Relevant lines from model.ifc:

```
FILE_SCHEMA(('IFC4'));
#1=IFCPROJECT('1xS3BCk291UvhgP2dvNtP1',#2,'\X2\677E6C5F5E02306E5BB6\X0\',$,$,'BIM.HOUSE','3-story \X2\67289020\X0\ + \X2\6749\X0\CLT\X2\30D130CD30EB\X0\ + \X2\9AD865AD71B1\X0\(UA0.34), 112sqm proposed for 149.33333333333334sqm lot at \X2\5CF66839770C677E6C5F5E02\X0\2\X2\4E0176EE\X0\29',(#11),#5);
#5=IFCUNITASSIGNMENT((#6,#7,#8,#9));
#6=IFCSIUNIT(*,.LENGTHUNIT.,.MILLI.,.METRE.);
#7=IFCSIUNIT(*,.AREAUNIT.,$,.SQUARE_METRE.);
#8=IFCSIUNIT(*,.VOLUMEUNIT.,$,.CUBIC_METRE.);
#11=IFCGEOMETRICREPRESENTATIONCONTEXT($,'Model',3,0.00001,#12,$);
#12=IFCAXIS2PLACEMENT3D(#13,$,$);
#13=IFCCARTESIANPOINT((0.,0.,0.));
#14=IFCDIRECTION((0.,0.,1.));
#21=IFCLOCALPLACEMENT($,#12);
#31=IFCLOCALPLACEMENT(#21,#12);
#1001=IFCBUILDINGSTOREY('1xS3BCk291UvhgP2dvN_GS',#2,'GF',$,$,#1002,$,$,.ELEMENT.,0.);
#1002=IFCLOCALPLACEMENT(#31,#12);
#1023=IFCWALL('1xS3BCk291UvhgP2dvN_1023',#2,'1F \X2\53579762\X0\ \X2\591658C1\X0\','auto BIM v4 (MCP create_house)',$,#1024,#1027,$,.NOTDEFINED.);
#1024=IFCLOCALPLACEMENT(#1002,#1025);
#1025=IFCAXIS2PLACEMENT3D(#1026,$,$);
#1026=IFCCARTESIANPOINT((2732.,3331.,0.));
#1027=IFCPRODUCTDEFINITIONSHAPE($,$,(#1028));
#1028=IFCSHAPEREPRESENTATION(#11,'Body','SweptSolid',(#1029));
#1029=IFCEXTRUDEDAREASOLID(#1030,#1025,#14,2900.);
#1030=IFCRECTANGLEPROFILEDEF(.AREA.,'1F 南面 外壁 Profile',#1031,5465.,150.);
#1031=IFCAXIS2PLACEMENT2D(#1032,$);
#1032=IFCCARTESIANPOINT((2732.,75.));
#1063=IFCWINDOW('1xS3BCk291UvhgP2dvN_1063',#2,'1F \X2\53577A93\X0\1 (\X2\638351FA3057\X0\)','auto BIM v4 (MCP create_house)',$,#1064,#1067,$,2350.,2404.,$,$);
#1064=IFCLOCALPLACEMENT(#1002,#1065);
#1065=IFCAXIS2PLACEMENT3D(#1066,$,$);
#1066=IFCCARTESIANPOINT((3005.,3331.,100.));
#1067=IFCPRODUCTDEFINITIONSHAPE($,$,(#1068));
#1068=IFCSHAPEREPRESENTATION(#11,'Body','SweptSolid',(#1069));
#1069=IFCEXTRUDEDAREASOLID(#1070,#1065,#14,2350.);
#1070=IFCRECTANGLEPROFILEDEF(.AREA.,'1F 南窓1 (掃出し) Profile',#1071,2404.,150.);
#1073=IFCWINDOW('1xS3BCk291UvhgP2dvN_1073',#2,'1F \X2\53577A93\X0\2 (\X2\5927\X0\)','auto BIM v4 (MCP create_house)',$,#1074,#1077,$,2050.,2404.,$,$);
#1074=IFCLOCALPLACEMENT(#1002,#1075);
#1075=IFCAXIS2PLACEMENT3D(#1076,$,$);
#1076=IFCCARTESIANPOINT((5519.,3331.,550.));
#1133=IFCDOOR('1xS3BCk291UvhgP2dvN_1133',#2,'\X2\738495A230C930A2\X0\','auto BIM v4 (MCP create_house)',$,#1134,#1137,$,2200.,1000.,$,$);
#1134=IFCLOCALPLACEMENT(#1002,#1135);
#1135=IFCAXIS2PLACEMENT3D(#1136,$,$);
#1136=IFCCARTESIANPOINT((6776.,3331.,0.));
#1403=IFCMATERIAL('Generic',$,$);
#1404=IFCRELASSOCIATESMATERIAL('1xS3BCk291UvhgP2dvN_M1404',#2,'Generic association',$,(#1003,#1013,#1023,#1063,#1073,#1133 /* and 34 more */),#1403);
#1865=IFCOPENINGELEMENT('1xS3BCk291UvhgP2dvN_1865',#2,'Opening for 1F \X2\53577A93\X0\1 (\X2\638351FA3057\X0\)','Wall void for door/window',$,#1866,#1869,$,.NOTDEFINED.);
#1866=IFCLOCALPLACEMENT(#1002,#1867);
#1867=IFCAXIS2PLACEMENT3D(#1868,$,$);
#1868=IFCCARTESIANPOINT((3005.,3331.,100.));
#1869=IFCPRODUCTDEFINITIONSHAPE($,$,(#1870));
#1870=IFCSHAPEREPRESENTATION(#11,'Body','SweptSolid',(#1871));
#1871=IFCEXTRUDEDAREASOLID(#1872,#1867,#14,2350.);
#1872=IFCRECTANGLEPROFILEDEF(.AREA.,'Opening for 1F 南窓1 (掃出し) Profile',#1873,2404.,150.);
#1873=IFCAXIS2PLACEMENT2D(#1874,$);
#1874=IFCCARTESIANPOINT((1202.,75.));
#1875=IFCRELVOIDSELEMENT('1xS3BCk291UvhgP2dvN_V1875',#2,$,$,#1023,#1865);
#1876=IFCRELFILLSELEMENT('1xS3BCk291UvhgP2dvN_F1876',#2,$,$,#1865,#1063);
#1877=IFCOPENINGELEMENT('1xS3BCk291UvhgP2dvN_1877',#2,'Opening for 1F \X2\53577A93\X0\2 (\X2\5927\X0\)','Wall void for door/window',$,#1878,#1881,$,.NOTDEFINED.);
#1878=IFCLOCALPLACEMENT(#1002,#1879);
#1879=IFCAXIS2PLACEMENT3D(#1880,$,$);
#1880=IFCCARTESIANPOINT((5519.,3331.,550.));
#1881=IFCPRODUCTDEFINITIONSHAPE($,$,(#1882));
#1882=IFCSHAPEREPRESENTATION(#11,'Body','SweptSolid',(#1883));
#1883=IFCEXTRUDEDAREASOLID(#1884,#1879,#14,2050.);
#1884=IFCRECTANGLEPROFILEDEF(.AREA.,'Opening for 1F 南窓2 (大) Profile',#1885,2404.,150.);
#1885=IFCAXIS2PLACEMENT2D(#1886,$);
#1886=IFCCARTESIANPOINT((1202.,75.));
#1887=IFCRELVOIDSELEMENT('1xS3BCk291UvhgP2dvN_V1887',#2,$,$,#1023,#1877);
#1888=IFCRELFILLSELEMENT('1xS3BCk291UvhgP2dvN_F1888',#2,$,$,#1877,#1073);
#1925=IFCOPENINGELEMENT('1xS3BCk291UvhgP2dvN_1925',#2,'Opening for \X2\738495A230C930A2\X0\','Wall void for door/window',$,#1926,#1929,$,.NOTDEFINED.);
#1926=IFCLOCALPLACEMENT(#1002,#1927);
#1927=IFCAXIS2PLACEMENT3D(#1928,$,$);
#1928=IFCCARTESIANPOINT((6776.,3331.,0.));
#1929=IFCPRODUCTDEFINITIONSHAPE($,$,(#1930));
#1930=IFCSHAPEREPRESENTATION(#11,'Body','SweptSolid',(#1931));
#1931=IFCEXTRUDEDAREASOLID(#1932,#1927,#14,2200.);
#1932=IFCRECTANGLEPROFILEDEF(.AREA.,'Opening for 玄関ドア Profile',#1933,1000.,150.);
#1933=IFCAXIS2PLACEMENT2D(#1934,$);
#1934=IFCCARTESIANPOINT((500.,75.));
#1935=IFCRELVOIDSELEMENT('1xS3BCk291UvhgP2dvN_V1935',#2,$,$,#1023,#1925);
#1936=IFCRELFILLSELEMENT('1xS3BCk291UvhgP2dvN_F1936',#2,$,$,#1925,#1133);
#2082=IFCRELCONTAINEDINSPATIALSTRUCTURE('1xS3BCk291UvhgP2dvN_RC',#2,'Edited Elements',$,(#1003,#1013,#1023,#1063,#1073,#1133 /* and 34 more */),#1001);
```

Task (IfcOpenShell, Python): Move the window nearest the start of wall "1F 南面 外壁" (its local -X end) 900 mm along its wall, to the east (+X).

```python
import ifcopenshell
import ifcopenshell.api.geometry
import ifcopenshell.util.placement

model = ifcopenshell.open("model.ifc")

window = model.by_guid("1xS3BCk291UvhgP2dvN_1063")
opening = window.FillsVoids[0].RelatingOpeningElement
wall = opening.VoidsElements[0].RelatingBuildingElement

wall_matrix = ifcopenshell.util.placement.get_local_placement(wall.ObjectPlacement)
shift = wall_matrix[:3, 0] * 900.0
before = ifcopenshell.util.placement.get_local_placement(window.ObjectPlacement)[:3, 3].copy()

# The window is not placed relative to its opening, so move both.
for product in (opening, window):
    matrix = ifcopenshell.util.placement.get_local_placement(product.ObjectPlacement)
    matrix[:3, 3] += shift
    ifcopenshell.api.geometry.edit_object_placement(model, product=product, matrix=matrix, is_si=False)

after = ifcopenshell.util.placement.get_local_placement(window.ObjectPlacement)[:3, 3]
print("window moved by", (after - before).round(3) + 0.0)

model.write("model_updated.ifc")
```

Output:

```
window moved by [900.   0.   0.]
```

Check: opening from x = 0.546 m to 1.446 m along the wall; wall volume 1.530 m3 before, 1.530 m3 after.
